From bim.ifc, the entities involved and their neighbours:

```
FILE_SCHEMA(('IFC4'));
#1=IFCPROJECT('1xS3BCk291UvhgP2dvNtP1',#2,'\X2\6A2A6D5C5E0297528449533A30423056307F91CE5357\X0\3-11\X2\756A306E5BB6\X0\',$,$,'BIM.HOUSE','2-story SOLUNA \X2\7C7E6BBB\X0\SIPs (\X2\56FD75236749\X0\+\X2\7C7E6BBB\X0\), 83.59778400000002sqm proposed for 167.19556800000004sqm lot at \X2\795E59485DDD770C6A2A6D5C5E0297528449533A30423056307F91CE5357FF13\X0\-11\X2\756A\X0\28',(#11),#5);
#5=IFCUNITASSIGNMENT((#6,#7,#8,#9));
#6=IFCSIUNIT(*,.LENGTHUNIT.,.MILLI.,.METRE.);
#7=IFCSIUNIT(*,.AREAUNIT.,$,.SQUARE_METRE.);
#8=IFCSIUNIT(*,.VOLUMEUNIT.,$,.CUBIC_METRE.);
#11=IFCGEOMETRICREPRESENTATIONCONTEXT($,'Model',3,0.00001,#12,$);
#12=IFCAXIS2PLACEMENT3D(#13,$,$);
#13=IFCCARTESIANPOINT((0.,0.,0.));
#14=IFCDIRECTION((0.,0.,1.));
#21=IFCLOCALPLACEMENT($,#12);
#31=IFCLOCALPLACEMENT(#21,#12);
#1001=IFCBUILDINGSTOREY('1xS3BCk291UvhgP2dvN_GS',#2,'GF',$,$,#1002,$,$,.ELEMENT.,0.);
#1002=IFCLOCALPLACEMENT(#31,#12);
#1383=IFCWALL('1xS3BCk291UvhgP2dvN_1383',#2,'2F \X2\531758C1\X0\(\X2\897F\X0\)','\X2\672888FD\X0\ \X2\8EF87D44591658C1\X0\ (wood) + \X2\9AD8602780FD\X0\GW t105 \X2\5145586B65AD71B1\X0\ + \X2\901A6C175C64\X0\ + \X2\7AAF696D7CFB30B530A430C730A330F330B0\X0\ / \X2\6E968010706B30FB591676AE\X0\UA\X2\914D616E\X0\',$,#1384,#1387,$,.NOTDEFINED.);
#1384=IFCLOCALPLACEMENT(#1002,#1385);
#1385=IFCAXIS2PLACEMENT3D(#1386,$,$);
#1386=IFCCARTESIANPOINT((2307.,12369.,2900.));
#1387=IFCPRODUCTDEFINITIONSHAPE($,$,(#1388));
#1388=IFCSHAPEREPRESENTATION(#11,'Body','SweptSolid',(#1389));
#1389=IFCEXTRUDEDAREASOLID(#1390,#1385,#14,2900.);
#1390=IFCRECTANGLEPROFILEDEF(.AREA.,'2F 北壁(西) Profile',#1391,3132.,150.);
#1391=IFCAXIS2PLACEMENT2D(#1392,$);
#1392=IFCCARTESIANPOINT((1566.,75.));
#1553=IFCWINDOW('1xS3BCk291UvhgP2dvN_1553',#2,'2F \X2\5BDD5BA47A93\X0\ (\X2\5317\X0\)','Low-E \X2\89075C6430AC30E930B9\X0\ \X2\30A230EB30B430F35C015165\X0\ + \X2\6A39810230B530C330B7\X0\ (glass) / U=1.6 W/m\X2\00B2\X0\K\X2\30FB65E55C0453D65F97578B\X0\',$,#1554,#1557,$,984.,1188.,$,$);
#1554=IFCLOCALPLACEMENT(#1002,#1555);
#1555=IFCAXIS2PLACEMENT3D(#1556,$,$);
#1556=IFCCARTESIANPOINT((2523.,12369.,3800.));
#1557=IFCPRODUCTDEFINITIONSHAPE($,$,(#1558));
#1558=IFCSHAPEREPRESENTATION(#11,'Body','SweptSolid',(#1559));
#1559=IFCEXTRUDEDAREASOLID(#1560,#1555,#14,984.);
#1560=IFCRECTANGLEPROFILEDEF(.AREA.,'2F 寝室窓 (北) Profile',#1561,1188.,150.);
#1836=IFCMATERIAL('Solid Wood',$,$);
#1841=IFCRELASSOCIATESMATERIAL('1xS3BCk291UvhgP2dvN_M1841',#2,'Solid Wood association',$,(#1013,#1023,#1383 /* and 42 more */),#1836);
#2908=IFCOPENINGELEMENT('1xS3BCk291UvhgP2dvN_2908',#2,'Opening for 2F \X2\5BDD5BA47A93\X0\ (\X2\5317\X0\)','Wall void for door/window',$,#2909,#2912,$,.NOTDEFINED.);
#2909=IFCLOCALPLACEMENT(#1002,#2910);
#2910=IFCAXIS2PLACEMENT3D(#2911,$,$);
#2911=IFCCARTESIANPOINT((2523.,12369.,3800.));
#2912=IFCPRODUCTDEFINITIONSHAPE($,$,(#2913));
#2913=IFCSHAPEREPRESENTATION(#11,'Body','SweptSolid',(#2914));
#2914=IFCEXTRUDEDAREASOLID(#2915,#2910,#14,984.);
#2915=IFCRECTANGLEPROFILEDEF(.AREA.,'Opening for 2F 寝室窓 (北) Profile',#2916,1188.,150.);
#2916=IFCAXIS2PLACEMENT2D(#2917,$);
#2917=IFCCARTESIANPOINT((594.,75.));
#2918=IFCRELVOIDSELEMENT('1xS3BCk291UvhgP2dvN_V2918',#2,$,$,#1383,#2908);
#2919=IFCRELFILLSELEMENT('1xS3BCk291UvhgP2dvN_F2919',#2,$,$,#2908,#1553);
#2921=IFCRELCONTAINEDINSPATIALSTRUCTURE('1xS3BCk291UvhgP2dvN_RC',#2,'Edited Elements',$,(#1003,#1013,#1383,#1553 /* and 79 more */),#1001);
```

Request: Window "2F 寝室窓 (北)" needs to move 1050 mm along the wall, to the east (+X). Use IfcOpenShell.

```python
import ifcopenshell
import ifcopenshell.api.geometry
import ifcopenshell.util.placement

model = ifcopenshell.open("bim.ifc")

window = model.by_guid("1xS3BCk291UvhgP2dvN_1553")
opening = window.FillsVoids[0].RelatingOpeningElement
wall = opening.VoidsElements[0].RelatingBuildingElement

wall_matrix = ifcopenshell.util.placement.get_local_placement(wall.ObjectPlacement)
shift = wall_matrix[:3, 0] * 1050.0
before = ifcopenshell.util.placement.get_local_placement(window.ObjectPlacement)[:3, 3].copy()

# The window is not placed relative to its opening, so move both.
for product in (opening, window):
    matrix = ifcopenshell.util.placement.get_local_placement(product.ObjectPlacement)
    matrix[:3, 3] += shift
    ifcopenshell.api.geometry.edit_object_placement(model, product=product, matrix=matrix, is_si=False)

after = ifcopenshell.util.placement.get_local_placement(window.ObjectPlacement)[:3, 3]
print("window moved by", (after - before).round(3) + 0.0)

model.write("bim_rev.ifc")
```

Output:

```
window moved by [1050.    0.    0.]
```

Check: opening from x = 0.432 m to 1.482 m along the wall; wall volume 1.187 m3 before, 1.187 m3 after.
